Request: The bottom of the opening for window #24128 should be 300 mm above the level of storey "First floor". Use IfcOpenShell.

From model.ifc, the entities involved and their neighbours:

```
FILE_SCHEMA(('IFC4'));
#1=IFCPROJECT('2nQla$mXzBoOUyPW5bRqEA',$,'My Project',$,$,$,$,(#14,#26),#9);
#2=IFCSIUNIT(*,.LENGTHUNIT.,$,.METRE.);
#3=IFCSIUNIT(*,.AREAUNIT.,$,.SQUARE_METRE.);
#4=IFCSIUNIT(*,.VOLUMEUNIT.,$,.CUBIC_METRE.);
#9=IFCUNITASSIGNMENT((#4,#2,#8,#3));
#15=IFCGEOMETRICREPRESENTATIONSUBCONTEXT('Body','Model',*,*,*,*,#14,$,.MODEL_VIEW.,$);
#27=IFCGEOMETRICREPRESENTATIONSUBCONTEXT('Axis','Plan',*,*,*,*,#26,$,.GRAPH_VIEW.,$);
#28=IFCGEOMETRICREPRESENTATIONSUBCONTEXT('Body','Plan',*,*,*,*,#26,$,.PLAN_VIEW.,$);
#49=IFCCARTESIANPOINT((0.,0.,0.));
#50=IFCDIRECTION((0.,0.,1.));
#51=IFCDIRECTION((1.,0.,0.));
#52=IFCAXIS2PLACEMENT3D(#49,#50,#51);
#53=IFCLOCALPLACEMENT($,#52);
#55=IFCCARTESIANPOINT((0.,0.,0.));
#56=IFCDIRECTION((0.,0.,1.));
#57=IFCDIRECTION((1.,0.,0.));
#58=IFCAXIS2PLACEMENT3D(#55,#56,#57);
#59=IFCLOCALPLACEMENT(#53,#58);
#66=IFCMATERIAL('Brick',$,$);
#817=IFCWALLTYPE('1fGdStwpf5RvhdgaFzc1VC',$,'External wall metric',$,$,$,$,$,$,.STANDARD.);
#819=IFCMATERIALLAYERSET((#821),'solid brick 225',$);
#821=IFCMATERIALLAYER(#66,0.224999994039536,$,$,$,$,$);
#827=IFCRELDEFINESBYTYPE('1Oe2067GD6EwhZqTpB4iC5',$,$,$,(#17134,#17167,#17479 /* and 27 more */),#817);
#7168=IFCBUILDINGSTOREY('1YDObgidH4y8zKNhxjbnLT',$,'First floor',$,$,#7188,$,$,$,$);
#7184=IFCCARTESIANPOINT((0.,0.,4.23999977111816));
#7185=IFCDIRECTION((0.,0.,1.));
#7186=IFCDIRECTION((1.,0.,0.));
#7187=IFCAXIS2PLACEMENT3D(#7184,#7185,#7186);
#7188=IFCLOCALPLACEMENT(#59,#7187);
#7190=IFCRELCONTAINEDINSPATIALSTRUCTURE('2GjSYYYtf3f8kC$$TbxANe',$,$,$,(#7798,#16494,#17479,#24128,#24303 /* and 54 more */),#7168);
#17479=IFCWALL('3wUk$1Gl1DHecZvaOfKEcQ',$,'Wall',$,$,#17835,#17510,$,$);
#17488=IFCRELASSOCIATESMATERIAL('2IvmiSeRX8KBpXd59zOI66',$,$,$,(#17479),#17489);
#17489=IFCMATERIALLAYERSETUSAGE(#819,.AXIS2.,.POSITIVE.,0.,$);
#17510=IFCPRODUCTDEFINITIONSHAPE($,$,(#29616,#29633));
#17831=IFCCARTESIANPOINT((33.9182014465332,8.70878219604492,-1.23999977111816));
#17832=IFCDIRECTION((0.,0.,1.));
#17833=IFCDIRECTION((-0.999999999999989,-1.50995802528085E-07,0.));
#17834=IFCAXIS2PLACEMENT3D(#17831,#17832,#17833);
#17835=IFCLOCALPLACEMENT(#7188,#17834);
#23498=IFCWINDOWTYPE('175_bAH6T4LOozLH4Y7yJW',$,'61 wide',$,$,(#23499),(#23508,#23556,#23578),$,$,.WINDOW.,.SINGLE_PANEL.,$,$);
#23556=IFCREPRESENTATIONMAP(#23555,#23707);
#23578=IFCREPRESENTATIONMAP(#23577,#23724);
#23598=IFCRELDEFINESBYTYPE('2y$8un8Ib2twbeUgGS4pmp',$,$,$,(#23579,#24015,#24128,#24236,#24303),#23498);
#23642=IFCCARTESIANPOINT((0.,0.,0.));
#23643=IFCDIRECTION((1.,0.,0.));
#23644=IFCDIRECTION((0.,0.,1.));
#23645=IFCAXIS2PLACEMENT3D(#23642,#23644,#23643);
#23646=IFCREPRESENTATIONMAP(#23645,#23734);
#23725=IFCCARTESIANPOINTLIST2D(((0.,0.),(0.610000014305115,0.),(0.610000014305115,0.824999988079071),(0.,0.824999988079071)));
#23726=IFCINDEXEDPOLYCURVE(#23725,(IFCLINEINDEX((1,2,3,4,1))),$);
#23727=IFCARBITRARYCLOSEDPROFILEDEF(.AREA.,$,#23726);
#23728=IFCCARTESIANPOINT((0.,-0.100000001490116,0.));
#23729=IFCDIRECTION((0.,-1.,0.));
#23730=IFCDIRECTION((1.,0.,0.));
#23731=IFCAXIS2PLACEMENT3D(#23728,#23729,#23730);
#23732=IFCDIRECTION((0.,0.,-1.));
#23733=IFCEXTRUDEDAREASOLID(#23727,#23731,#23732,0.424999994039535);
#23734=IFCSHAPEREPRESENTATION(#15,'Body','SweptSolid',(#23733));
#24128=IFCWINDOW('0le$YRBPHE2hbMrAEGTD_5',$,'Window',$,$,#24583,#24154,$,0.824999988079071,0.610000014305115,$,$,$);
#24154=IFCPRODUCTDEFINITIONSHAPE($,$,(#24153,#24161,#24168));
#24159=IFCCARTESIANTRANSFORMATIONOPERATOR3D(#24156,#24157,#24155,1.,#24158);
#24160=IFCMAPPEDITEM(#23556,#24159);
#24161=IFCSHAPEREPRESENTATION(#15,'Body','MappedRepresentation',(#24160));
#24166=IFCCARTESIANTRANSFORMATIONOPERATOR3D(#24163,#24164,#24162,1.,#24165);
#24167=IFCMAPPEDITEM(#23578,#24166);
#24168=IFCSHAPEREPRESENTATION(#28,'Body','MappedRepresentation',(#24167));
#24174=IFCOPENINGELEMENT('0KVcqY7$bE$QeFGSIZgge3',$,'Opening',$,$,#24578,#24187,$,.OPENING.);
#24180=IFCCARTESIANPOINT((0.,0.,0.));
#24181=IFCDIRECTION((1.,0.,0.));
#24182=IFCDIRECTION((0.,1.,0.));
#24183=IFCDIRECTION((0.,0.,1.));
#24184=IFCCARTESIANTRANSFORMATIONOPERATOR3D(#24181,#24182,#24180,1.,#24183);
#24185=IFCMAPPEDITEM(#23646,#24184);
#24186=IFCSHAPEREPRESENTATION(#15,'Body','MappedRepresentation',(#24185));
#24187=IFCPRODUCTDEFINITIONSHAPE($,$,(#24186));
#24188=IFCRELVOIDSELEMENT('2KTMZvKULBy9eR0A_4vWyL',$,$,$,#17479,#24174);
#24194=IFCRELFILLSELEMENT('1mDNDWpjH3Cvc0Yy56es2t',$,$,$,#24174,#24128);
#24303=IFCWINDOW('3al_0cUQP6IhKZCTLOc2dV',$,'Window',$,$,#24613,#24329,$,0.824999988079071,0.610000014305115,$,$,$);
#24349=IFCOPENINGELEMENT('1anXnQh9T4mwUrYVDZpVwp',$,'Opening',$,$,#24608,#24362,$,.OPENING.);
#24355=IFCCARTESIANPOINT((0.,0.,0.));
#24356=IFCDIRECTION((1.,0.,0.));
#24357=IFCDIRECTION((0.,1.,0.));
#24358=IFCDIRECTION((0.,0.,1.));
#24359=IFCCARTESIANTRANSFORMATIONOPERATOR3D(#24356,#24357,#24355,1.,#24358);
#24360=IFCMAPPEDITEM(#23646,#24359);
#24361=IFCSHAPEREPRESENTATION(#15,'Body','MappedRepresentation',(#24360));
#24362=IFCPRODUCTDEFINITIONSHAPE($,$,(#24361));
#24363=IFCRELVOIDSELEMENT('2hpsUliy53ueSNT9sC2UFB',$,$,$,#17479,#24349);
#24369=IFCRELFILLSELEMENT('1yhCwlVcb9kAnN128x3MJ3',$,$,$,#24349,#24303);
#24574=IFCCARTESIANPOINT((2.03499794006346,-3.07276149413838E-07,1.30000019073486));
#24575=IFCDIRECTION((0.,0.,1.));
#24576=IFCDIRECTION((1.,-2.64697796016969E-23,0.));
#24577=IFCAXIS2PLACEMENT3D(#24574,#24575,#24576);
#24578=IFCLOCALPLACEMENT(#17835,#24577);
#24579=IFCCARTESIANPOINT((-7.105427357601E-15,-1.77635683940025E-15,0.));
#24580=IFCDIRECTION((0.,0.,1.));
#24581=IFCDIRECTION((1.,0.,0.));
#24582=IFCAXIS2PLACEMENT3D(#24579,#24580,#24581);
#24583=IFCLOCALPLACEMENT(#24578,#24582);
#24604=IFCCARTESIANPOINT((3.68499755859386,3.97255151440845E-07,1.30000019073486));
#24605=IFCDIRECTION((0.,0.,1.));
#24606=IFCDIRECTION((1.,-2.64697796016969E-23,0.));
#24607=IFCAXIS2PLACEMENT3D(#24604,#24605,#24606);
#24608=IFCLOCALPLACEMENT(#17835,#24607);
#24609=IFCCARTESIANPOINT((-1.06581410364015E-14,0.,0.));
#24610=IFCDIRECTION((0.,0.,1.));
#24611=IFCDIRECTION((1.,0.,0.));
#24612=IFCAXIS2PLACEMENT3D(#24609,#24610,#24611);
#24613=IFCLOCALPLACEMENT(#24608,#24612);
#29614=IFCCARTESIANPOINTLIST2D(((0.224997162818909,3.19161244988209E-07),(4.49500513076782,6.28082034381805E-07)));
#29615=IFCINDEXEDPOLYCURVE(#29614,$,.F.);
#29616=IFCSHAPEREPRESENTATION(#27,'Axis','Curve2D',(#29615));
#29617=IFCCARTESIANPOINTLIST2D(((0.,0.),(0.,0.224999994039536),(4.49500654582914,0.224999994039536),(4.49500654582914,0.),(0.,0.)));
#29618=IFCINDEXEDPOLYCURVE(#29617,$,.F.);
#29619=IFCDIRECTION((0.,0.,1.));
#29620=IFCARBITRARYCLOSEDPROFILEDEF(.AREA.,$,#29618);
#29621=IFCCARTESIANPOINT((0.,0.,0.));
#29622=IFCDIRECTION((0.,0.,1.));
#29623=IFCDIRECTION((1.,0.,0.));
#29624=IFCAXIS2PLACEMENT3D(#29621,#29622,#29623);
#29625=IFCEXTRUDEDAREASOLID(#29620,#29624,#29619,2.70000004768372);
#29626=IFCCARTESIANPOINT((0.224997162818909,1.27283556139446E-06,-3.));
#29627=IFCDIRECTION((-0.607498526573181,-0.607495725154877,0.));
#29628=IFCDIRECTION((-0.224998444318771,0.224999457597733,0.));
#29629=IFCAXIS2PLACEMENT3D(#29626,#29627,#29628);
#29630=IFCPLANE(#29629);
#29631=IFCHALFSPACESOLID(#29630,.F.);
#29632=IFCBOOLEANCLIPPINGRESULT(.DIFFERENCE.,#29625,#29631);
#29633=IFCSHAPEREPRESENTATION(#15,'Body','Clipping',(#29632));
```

```python
import numpy as np
import ifcopenshell
import ifcopenshell.api.geometry
import ifcopenshell.geom
import ifcopenshell.util.element
import ifcopenshell.util.placement
import ifcopenshell.util.shape
import ifcopenshell.util.unit

model = ifcopenshell.open("model.ifc")
unit_scale = ifcopenshell.util.unit.calculate_unit_scale(model)

window = model.by_guid("0le$YRBPHE2hbMrAEGTD_5")
opening = window.FillsVoids[0].RelatingOpeningElement
storey = ifcopenshell.util.element.get_container(window, ifc_class="IfcBuildingStorey")
level = ifcopenshell.util.placement.get_local_placement(storey.ObjectPlacement)[2, 3]

# The opening's origin need not be at the sill, so measure its lowest point.
shape = ifcopenshell.geom.create_shape(ifcopenshell.geom.settings(), opening)
bottom = ifcopenshell.util.shape.get_shape_bottom_elevation(shape, shape.geometry) / unit_scale
dz = level + 0.3 - bottom

shift = np.array([0.0, 0.0, dz])
# The window is placed relative to its opening, so it follows when the opening moves.
matrix = ifcopenshell.util.placement.get_local_placement(opening.ObjectPlacement)
matrix[:3, 3] += shift
ifcopenshell.api.geometry.edit_object_placement(
    model, product=opening, matrix=matrix, is_si=False, should_transform_children=True
)

print(f"moved by {dz * unit_scale:+.3f} m")

model.write("model-out.ifc")
```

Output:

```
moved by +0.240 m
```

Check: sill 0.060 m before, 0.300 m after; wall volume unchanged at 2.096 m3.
